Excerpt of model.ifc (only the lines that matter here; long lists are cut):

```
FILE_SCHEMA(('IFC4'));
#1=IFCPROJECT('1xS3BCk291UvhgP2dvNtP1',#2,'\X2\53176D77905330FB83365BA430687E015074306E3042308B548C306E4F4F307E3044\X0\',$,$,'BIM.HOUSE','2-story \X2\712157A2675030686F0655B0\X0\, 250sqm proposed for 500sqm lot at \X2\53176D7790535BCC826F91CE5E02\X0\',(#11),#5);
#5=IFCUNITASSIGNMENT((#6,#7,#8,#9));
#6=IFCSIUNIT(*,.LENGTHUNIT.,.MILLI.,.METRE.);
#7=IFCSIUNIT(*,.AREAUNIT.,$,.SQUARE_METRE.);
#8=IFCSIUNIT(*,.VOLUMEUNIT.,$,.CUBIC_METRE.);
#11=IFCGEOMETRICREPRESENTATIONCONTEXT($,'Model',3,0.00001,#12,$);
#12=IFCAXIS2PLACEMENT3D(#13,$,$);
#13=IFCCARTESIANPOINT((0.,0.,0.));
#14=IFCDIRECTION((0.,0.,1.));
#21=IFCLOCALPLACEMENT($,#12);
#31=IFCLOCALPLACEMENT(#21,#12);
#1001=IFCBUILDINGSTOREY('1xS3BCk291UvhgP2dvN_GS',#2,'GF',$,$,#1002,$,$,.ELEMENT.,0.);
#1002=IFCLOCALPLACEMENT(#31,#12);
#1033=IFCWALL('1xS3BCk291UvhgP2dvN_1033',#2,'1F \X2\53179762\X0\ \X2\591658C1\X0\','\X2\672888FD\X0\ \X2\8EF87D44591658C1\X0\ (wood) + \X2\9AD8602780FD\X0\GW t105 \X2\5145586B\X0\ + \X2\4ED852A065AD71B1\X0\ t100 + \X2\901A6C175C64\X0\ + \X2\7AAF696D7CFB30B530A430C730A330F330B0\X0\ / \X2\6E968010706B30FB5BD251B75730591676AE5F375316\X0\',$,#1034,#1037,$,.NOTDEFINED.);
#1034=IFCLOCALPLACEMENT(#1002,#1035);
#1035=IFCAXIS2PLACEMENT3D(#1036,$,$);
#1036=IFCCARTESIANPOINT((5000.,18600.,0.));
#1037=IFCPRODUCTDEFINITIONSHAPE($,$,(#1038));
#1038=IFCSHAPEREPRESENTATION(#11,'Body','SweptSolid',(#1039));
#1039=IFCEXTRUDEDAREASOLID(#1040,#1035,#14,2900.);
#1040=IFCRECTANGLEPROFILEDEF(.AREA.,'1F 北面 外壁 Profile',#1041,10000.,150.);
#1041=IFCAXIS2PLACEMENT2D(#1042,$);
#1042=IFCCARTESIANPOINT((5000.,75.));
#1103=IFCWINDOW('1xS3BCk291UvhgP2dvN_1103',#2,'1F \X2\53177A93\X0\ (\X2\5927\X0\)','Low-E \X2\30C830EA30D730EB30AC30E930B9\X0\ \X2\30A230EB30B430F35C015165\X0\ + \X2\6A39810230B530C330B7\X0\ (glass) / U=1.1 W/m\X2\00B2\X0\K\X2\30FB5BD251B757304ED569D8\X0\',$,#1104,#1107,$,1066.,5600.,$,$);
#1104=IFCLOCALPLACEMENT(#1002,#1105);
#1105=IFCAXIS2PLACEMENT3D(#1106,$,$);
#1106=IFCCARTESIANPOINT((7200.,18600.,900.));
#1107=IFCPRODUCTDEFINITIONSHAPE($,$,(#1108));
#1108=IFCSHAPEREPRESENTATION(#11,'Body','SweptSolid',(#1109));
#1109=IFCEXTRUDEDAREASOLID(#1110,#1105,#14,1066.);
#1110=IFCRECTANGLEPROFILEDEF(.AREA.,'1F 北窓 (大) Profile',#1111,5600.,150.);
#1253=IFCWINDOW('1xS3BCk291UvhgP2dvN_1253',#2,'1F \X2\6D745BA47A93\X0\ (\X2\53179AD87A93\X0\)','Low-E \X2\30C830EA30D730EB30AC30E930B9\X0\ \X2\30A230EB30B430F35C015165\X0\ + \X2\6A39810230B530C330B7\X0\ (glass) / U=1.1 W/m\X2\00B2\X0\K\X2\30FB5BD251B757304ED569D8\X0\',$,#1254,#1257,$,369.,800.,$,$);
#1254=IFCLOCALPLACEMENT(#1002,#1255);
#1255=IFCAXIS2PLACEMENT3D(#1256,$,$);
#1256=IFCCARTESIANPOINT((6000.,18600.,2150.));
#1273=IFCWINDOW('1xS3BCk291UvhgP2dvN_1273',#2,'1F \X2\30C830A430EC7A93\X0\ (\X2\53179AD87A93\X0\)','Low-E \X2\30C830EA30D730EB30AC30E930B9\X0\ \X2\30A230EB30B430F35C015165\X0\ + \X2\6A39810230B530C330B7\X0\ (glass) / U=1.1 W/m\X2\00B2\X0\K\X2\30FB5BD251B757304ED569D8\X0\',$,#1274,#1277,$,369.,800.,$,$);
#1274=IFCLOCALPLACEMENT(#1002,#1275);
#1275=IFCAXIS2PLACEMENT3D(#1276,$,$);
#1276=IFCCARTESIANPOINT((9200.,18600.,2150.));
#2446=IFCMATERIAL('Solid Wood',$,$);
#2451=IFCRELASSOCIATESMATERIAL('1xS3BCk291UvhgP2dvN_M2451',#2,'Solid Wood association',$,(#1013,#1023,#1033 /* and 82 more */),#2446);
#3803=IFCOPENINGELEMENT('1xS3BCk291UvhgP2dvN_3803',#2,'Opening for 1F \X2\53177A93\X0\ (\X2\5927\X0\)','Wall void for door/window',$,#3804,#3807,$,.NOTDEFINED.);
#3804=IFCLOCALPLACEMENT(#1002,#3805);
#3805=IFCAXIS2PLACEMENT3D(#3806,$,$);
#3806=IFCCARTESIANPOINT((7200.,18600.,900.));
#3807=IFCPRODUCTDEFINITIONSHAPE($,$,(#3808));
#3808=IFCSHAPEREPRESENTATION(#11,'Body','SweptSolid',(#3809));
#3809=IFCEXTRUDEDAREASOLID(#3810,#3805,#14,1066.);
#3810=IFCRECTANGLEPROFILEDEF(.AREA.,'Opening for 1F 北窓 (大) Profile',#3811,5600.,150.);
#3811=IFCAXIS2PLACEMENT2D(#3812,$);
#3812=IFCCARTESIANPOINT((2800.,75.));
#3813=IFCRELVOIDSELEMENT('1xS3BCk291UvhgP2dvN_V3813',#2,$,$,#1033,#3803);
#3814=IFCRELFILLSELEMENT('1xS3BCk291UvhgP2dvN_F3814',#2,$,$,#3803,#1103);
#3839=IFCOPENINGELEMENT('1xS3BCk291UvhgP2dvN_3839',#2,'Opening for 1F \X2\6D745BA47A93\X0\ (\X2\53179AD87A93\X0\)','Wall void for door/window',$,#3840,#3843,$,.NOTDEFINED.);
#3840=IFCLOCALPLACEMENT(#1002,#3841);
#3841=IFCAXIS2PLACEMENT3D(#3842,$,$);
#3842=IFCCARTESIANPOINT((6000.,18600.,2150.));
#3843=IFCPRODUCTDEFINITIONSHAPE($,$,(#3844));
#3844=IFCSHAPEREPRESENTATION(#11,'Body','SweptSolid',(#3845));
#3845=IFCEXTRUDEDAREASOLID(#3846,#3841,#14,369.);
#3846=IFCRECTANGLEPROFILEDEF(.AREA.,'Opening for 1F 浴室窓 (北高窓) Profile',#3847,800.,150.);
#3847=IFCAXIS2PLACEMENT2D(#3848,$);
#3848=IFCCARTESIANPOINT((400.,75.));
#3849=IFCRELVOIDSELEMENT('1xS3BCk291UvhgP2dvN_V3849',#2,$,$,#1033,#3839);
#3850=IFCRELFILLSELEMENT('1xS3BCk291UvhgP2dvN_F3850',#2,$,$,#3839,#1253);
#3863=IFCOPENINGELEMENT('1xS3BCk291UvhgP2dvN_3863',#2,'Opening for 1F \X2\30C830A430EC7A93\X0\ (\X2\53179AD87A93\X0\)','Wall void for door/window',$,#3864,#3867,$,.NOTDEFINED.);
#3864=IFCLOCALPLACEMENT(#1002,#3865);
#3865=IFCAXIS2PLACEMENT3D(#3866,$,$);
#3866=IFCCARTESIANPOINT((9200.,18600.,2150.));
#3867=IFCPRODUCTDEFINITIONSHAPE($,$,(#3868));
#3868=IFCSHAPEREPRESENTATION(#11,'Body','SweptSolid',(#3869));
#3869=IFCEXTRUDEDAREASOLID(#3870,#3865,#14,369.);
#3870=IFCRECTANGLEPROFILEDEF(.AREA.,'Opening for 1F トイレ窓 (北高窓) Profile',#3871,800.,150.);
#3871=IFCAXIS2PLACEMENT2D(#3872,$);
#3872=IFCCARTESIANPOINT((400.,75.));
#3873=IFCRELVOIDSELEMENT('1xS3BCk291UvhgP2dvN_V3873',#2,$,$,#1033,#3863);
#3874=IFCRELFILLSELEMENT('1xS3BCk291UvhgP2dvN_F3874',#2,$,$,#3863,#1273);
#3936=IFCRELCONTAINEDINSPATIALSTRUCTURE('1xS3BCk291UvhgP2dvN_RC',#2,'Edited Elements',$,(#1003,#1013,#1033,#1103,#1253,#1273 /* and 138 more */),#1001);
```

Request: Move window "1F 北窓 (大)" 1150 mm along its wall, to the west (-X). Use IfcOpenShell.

```python
import ifcopenshell
import ifcopenshell.api.geometry
import ifcopenshell.util.placement
import ifcopenshell.util.unit

model = ifcopenshell.open("model.ifc")
unit_scale = ifcopenshell.util.unit.calculate_unit_scale(model)

window = model.by_guid("1xS3BCk291UvhgP2dvN_1103")
opening = window.FillsVoids[0].RelatingOpeningElement
wall = opening.VoidsElements[0].RelatingBuildingElement

wall_matrix = ifcopenshell.util.placement.get_local_placement(wall.ObjectPlacement)
shift = wall_matrix[:3, 0] * -1.15 / unit_scale
before = ifcopenshell.util.placement.get_local_placement(window.ObjectPlacement)[:3, 3].copy()

# The window is not placed relative to its opening, so move both.
for product in (opening, window):
    matrix = ifcopenshell.util.placement.get_local_placement(product.ObjectPlacement)
    matrix[:3, 3] += shift
    ifcopenshell.api.geometry.edit_object_placement(model, product=product, matrix=matrix, is_si=False)

after = ifcopenshell.util.placement.get_local_placement(window.ObjectPlacement)[:3, 3]
print("window moved by", (after - before).round(3) + 0.0)

model.write("model_updated.ifc")
```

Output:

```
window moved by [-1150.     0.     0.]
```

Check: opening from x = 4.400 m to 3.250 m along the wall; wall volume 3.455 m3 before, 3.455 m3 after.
